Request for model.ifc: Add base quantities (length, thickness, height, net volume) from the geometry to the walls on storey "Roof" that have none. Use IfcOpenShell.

First a look at what the model holds.

```python
import ifcopenshell
import ifcopenshell.util.element
import ifcopenshell.util.unit

model = ifcopenshell.open("model.ifc")
print(model.schema)
for unit_type in ("LENGTHUNIT", "AREAUNIT", "VOLUMEUNIT"):
    print(unit_type, ifcopenshell.util.unit.calculate_unit_scale(model, unit_type))
storey = next(s for s in model.by_type("IfcBuildingStorey") if s.Name == "Roof")
walls = [e for e in ifcopenshell.util.element.get_decomposition(storey) if e.is_a("IfcWall")]
for e in sorted(walls, key=lambda e: e.id()):
    print(e.id(), e.is_a(), e.Name, list(ifcopenshell.util.element.get_psets(e, qtos_only=True)), sep=" | ")
```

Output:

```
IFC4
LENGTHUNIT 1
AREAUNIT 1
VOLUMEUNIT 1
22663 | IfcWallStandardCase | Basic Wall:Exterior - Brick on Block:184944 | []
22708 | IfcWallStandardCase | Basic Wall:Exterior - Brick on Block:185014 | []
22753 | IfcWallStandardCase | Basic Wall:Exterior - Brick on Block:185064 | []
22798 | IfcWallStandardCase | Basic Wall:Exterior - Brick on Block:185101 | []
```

```python
import ifcopenshell
import ifcopenshell.api.pset
import ifcopenshell.geom
import ifcopenshell.util.element
import ifcopenshell.util.shape
import ifcopenshell.util.unit

model = ifcopenshell.open("model.ifc")
unit_scale = ifcopenshell.util.unit.calculate_unit_scale(model)
volume_scale = ifcopenshell.util.unit.calculate_unit_scale(model, "VOLUMEUNIT")
settings = ifcopenshell.geom.settings()

storey = next(s for s in model.by_type("IfcBuildingStorey") if s.Name == "Roof")
walls = [e for e in ifcopenshell.util.element.get_decomposition(storey) if e.is_a("IfcWall")]

for e in sorted(walls, key=lambda e: e.id()):
    if ifcopenshell.util.element.get_psets(e, qtos_only=True, should_inherit=False):
        continue
    # Geometry comes back in metres, in the element's own axes.
    shape = ifcopenshell.geom.create_shape(settings, e)
    values = {
        "Length": ifcopenshell.util.shape.get_x(shape.geometry) / unit_scale,
        "Width": ifcopenshell.util.shape.get_y(shape.geometry) / unit_scale,
        "Height": ifcopenshell.util.shape.get_z(shape.geometry) / unit_scale,
        "NetVolume": ifcopenshell.util.shape.get_volume(shape.geometry) / volume_scale,
    }
    qto = ifcopenshell.api.pset.add_qto(model, product=e, name="Qto_WallBaseQuantities")
    ifcopenshell.api.pset.edit_qto(model, qto=qto, properties=values)
    print(e.id(), {k: round(v, 3) for k, v in values.items()})

model.write("model_updated.ifc")
```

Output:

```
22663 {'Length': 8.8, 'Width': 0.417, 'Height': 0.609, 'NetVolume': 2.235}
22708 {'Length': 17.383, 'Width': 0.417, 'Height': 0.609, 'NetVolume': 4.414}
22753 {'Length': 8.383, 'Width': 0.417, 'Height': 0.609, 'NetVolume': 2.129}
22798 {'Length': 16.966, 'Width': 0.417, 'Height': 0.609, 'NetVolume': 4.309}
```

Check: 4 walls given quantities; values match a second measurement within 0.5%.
